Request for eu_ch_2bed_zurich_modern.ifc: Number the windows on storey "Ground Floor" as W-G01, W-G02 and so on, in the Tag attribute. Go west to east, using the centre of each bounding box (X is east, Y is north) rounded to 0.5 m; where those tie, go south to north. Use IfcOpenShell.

First a look at what the model holds.

```python
import ifcopenshell
import ifcopenshell.util.element
import ifcopenshell.util.placement

model = ifcopenshell.open("eu_ch_2bed_zurich_modern.ifc")
print(model.schema)
storey = next(s for s in model.by_type("IfcBuildingStorey") if s.Name == "Ground Floor")
windows = [e for e in ifcopenshell.util.element.get_decomposition(storey) if e.is_a("IfcWindow")]
for e in sorted(windows, key=lambda e: e.id()):
    origin = ifcopenshell.util.placement.get_local_placement(e.ObjectPlacement)[:3, 3]
    print(e.id(), e.Tag, e.Name, origin.round(2) + 0.0, sep=" | ")
```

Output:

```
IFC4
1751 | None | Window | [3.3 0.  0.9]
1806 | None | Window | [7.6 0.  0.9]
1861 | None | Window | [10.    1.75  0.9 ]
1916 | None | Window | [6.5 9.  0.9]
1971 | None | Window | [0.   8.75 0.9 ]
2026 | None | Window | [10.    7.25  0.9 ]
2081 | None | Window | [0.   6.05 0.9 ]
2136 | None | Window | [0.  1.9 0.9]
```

```python
import ifcopenshell
import ifcopenshell.geom
import ifcopenshell.util.element
import ifcopenshell.util.shape

model = ifcopenshell.open("eu_ch_2bed_zurich_modern.ifc")
settings = ifcopenshell.geom.settings()
settings.set("use-world-coords", True)


def centre(element):
    shape = ifcopenshell.geom.create_shape(settings, element)
    return ifcopenshell.util.shape.get_bbox_centroid(shape.geometry)


storey = next(s for s in model.by_type("IfcBuildingStorey") if s.Name == "Ground Floor")
windows = [e for e in ifcopenshell.util.element.get_decomposition(storey) if e.is_a("IfcWindow")]

# Insertion points can sit at a corner or the storey origin, so sort by the geometry (in metres).
centres = {e: centre(e) for e in windows}
windows.sort(key=lambda e: (round(centres[e][0] / 0.5), centres[e][1]))

for i, e in enumerate(windows, start=1):
    number = f"W-G{i:02d}"
    e.Tag = number
    print(e.id(), number)

model.write("eu_ch_2bed_zurich_modern_rev.ifc")
```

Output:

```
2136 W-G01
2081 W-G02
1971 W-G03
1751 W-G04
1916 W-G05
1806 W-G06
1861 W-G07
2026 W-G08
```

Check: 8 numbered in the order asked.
